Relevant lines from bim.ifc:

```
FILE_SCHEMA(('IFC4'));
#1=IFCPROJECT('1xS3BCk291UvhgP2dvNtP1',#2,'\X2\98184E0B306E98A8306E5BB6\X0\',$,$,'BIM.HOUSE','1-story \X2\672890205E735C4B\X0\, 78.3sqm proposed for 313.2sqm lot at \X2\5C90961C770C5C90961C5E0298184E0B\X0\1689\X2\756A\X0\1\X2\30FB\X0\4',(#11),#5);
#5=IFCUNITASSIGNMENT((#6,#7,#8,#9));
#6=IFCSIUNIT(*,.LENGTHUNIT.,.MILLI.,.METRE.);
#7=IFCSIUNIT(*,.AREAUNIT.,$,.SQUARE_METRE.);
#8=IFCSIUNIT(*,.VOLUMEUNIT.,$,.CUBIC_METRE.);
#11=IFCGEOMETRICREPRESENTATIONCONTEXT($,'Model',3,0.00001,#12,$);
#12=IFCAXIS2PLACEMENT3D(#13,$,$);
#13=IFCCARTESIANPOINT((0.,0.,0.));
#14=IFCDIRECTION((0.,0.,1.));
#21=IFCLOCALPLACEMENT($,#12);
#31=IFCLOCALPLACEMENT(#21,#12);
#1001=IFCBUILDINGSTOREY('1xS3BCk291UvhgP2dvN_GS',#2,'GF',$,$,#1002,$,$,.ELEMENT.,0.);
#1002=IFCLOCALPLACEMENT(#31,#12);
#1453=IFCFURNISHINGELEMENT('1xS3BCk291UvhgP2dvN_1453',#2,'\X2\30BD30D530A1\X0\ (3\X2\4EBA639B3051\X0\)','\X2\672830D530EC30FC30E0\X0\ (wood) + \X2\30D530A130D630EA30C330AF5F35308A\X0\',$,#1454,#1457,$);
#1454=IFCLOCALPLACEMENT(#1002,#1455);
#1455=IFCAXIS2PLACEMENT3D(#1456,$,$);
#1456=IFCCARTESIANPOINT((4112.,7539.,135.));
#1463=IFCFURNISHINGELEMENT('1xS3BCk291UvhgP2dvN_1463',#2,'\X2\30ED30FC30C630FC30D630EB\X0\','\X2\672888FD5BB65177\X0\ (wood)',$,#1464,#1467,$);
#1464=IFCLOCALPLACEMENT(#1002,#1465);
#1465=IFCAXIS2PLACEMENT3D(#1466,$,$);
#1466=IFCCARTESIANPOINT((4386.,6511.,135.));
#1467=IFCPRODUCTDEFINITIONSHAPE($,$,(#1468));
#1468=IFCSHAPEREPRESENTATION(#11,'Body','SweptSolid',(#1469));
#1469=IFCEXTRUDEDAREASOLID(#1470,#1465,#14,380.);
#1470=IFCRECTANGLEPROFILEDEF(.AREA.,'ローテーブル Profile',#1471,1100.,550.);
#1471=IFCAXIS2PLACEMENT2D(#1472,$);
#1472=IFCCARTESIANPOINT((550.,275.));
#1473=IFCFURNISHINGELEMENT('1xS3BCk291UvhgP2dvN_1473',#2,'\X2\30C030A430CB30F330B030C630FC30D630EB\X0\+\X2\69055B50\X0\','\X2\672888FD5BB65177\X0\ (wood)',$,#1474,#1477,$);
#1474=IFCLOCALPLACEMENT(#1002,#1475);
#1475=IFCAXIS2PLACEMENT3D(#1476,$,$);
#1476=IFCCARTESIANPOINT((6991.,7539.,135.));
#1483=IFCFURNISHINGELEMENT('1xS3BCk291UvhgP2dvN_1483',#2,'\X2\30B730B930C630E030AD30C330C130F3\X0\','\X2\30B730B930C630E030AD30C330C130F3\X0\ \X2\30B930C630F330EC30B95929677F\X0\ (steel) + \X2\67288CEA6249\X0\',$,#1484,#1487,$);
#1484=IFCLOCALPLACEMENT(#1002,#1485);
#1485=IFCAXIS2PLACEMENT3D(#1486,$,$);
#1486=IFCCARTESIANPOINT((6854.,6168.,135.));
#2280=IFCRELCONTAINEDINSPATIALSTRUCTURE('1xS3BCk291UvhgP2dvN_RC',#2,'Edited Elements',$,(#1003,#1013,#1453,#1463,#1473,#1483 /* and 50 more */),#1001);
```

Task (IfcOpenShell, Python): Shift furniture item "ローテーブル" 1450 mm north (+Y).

```python
import ifcopenshell
import ifcopenshell.api.geometry
import ifcopenshell.util.placement
import ifcopenshell.util.unit

model = ifcopenshell.open("bim.ifc")
unit_scale = ifcopenshell.util.unit.calculate_unit_scale(model)

item = model.by_guid("1xS3BCk291UvhgP2dvN_1463")
matrix = ifcopenshell.util.placement.get_local_placement(item.ObjectPlacement)
matrix[1, 3] += 1.45 / unit_scale
ifcopenshell.api.geometry.edit_object_placement(model, product=item, matrix=matrix, is_si=False)

print(ifcopenshell.util.placement.get_local_placement(item.ObjectPlacement).round(3) + 0.0)

model.write("bim_edited.ifc")
```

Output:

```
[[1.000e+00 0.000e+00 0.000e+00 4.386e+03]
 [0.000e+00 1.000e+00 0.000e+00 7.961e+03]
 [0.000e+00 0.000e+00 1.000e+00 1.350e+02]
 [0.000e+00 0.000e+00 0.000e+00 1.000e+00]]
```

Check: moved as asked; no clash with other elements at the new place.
